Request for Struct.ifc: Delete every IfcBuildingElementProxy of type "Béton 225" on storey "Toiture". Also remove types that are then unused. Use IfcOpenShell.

First a look at what the model holds.

```python
import ifcopenshell
import ifcopenshell.util.element

model = ifcopenshell.open("Struct.ifc")
print(model.schema)
storey = next(s for s in model.by_type("IfcBuildingStorey") if s.Name == "Toiture")
proxies = [e for e in ifcopenshell.util.element.get_decomposition(storey) if e.is_a("IfcBuildingElementProxy")]
seen = {}
for e in proxies:
    element_type = ifcopenshell.util.element.get_type(e)
    name = element_type.Name if element_type not in (None, e) else None
    seen[name] = seen.get(name, 0) + 1
for name, count in sorted(seen.items(), key=str):
    print(count, "x", name)
```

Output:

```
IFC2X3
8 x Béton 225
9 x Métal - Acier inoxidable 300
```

```python
import ifcopenshell
import ifcopenshell.api.root
import ifcopenshell.util.element

model = ifcopenshell.open("Struct.ifc")

storey = next(s for s in model.by_type("IfcBuildingStorey") if s.Name == "Toiture")
proxies = [e for e in ifcopenshell.util.element.get_decomposition(storey) if e.is_a("IfcBuildingElementProxy")]
targets = [e for e in proxies if (t := ifcopenshell.util.element.get_type(e)) not in (None, e) and t.Name == "Béton 225"]
types = {ifcopenshell.util.element.get_type(e) for e in targets} - {None, *targets}

for e in targets:
    ifcopenshell.api.root.remove_product(model, product=e)
print(len(targets), "removed")

unused = [t for t in types if not ifcopenshell.util.element.get_types(t)]
for t in unused:
    ifcopenshell.api.root.remove_product(model, product=t)
print(len(unused), "unused types removed")

model.write("Struct_edited.ifc")
```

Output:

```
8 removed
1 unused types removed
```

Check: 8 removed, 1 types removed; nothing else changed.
